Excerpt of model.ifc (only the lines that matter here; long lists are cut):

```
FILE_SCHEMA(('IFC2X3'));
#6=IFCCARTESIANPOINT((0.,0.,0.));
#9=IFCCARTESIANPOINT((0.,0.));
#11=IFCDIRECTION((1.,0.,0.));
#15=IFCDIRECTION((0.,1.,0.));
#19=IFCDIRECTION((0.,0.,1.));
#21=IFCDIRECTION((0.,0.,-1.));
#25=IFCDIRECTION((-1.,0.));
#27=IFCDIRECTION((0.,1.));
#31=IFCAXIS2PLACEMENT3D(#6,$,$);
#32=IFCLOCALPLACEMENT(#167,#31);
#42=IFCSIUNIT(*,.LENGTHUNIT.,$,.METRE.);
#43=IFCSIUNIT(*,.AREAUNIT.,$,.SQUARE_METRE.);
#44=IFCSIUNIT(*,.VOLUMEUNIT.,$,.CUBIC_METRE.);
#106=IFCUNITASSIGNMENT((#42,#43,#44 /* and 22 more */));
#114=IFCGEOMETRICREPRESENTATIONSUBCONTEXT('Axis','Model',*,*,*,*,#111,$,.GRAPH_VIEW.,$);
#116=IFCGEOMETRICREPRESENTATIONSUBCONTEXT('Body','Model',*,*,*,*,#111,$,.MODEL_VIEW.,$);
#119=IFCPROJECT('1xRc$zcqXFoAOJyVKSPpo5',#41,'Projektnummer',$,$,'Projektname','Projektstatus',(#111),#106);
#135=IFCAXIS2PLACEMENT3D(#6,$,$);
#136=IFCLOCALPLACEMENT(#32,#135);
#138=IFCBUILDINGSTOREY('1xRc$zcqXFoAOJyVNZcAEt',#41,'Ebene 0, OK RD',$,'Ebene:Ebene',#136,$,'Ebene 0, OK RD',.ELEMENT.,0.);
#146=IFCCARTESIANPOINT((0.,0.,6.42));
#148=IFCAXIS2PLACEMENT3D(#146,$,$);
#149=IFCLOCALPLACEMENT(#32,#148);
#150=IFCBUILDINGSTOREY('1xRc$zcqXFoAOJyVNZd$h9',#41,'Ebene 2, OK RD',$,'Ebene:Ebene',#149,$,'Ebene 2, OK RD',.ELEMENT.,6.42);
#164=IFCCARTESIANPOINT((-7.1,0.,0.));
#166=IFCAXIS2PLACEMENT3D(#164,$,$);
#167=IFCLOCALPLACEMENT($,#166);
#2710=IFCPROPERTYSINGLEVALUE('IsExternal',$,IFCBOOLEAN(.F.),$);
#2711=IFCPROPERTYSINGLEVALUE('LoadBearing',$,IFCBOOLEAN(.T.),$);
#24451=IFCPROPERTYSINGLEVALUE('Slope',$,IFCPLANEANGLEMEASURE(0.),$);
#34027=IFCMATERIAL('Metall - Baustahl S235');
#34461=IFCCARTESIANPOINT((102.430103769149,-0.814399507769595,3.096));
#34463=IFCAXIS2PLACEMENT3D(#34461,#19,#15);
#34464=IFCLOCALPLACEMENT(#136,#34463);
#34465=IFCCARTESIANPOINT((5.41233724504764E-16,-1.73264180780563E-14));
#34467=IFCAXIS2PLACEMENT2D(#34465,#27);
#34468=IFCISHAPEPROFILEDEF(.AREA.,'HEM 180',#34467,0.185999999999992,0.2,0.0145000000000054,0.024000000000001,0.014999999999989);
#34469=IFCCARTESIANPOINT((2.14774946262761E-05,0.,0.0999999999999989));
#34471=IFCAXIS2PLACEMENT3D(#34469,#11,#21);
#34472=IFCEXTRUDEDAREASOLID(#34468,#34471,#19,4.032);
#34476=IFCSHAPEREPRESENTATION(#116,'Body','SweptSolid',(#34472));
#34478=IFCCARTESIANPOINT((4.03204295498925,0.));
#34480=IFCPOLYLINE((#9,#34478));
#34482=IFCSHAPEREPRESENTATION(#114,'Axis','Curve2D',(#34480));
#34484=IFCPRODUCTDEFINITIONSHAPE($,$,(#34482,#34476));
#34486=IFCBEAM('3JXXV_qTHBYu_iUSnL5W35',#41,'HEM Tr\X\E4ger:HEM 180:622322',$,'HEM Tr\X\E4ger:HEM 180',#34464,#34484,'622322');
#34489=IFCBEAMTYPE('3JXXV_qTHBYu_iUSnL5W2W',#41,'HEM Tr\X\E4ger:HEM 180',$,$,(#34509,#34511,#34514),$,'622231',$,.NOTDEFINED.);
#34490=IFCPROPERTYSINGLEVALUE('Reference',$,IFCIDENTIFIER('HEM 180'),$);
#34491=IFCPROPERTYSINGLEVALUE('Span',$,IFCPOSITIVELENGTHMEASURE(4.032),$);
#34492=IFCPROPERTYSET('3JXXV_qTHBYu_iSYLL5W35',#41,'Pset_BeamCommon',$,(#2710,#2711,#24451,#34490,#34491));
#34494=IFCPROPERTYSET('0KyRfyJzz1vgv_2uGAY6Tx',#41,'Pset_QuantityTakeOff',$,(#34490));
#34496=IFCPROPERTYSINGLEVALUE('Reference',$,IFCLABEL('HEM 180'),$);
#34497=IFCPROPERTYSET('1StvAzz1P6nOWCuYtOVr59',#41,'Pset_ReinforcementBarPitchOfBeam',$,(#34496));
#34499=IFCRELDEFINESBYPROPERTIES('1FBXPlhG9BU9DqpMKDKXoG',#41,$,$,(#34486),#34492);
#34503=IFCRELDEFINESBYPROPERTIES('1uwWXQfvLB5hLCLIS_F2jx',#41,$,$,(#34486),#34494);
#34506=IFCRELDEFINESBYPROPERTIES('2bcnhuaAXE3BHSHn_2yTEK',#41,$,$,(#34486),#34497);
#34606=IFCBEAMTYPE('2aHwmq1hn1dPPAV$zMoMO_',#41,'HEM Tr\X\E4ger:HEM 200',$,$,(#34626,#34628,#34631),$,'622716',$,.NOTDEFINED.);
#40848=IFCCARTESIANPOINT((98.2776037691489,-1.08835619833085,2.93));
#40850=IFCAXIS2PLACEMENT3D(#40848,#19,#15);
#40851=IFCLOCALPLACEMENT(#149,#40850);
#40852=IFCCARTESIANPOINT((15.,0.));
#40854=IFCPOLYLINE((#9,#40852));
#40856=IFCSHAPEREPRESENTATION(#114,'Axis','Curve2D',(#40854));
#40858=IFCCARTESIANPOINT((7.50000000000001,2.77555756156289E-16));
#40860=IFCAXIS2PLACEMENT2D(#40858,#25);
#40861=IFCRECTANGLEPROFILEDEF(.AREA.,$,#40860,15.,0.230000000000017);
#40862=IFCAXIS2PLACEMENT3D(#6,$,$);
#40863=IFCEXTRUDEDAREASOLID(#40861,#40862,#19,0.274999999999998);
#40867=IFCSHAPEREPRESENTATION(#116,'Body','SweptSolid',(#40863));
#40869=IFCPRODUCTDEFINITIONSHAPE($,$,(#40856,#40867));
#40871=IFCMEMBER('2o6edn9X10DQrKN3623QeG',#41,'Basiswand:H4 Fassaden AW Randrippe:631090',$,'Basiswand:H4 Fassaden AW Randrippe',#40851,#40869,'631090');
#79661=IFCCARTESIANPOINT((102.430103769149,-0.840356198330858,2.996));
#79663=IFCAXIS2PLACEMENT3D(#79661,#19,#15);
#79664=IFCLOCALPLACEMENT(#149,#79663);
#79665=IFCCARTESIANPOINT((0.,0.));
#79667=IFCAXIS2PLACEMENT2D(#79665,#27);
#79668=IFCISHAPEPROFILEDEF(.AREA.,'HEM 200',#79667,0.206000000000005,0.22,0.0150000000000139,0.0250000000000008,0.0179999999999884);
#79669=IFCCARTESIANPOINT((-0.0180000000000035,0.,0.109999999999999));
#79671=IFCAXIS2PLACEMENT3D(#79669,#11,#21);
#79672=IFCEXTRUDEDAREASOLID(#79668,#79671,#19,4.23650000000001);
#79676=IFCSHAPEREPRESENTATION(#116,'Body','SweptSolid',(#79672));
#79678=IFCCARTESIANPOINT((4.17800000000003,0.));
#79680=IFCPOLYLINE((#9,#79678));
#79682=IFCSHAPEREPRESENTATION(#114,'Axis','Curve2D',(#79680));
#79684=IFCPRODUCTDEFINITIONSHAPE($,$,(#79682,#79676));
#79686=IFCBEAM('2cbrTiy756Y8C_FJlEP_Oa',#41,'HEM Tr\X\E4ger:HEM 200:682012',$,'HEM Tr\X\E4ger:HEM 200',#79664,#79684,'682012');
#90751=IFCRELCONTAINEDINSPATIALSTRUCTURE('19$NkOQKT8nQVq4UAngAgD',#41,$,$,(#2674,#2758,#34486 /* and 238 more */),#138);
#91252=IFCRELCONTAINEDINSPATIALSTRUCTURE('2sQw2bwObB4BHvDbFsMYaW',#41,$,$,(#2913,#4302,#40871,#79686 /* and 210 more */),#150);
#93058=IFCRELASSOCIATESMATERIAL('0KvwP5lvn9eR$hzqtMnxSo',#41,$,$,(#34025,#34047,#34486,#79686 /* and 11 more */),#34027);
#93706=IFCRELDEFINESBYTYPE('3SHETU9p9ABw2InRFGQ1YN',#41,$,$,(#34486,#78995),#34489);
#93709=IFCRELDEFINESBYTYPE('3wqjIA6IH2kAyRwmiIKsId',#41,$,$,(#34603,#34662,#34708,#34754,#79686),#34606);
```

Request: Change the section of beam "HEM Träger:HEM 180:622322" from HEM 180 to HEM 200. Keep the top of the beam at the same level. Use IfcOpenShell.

```python
import ifcopenshell
import ifcopenshell.api.pset
import ifcopenshell.api.type
import ifcopenshell.util.element
import ifcopenshell.util.representation

model = ifcopenshell.open("model.ifc")

member = model.by_guid("3JXXV_qTHBYu_iUSnL5W35")
source = next(p for p in model.by_type("IfcIShapeProfileDef") if p.ProfileName == "HEM 200")

body = ifcopenshell.util.representation.get_representation(member, "Model", "Body")
solid = body.Items[0]
old_profile = solid.SweptArea

# Copy the section's sizes but keep this member's own profile position.
profile = ifcopenshell.util.element.copy(model, source)
# Profiles are centred, so shift by half the change in depth to hold the top.
shift = (old_profile.OverallDepth - profile.OverallDepth) / 2
x, y = old_profile.Position.Location.Coordinates
up = (-1.0, 0.0)  # upwards, in the solid's own plane
location = model.createIfcCartesianPoint((x + up[0] * shift, y + up[1] * shift))
profile.Position = model.createIfcAxis2Placement2D(location, old_profile.Position.RefDirection)
solid.SweptArea = profile
if not model.get_total_inverses(old_profile):
    ifcopenshell.util.element.remove_deep2(model, old_profile)

new_type = model.by_guid("2aHwmq1hn1dPPAV$zMoMO_")
ifcopenshell.api.type.assign_type(
    model, related_objects=[member], relating_type=new_type, should_map_representations=False
)
member.Name = member.Name.replace("HEM 180", "HEM 200")
member.ObjectType = "HEM Träger:HEM 200"
pset = model.by_id(ifcopenshell.util.element.get_pset(member, "Pset_BeamCommon", should_inherit=False)["id"])
ifcopenshell.api.pset.edit_pset(model, pset=pset, properties={"Reference": "HEM 200"})
pset = model.by_id(ifcopenshell.util.element.get_pset(member, "Pset_QuantityTakeOff", should_inherit=False)["id"])
ifcopenshell.api.pset.edit_pset(model, pset=pset, properties={"Reference": "HEM 200"})
pset = model.by_id(ifcopenshell.util.element.get_pset(member, "Pset_ReinforcementBarPitchOfBeam", should_inherit=False)["id"])
ifcopenshell.api.pset.edit_pset(model, pset=pset, properties={"Reference": "HEM 200"})

print(solid.SweptArea)

model.write("model_rev.ifc")
```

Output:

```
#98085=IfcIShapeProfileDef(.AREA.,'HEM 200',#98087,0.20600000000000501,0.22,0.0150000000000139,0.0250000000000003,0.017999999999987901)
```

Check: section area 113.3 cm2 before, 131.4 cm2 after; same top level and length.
